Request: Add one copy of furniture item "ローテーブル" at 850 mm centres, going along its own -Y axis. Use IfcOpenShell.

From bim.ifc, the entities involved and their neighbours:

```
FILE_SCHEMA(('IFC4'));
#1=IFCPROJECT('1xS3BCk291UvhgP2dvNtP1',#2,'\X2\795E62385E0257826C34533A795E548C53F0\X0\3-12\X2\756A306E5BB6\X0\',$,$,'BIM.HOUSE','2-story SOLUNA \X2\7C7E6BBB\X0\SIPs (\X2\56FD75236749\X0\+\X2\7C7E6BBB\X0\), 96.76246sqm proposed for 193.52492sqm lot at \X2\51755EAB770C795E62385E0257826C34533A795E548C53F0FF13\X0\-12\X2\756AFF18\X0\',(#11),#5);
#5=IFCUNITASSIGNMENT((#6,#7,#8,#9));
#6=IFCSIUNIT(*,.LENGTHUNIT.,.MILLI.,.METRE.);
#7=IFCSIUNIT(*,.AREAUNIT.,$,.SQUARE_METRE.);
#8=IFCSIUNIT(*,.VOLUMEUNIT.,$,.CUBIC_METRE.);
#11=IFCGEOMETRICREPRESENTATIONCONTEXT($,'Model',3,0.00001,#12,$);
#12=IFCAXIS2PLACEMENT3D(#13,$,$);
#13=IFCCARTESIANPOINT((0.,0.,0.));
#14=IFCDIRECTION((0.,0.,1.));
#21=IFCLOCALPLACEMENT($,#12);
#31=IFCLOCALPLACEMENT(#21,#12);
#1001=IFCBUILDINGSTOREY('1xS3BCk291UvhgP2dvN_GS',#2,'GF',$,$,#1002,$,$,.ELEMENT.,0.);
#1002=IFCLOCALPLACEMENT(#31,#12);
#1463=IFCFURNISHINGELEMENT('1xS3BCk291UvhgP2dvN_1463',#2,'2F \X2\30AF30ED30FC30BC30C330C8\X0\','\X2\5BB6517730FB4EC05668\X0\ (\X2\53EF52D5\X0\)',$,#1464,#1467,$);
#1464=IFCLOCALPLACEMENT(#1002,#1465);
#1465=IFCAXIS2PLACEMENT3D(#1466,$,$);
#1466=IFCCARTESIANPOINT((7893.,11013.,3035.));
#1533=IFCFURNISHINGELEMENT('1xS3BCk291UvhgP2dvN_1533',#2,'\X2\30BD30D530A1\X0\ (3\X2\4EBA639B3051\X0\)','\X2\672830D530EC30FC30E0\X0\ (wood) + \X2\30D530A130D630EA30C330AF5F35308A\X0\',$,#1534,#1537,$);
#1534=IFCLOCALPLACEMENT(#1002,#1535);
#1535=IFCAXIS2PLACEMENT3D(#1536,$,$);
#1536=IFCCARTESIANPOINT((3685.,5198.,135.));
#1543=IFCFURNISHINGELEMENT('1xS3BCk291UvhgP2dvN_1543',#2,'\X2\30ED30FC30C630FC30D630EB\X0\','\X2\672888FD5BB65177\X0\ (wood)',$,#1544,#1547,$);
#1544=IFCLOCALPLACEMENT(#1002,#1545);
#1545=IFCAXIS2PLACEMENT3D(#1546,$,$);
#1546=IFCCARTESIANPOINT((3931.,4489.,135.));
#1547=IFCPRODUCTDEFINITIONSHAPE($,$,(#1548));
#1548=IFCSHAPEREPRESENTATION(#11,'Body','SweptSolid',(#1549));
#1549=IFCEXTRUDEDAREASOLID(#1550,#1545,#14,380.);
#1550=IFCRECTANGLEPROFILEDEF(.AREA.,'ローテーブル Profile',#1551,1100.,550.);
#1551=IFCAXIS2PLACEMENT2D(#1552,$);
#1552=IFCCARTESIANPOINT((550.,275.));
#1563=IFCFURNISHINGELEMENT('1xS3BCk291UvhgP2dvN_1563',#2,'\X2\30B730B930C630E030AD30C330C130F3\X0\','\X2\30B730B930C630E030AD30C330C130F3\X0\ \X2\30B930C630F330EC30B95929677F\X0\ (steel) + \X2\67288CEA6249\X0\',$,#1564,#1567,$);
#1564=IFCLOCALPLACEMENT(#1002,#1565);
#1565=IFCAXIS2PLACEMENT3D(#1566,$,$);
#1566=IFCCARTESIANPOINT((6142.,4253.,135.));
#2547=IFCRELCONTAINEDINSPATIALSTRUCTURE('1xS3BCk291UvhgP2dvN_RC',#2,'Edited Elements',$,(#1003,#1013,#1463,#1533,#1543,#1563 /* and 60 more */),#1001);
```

```python
import ifcopenshell
import ifcopenshell.api.geometry
import ifcopenshell.api.root
import ifcopenshell.util.element
import ifcopenshell.util.placement
import ifcopenshell.util.unit

model = ifcopenshell.open("bim.ifc")
unit_scale = ifcopenshell.util.unit.calculate_unit_scale(model)


def reuse_history(source, copy):
    """copy_class also copies each property set's owner history, people and application; keep the originals."""
    for rel in copy.IsDefinedBy:
        if rel.is_a("IfcRelDefinesByProperties") and (history := rel.RelatingPropertyDefinition.OwnerHistory):
            rel.RelatingPropertyDefinition.OwnerHistory = source.OwnerHistory
            ifcopenshell.util.element.remove_deep2(model, history)


source = model.by_id(1543)
base = ifcopenshell.util.placement.get_local_placement(source.ObjectPlacement)
step = -base[:3, 1] * 0.85 / unit_scale

for i in range(1, 2):
    copy = ifcopenshell.api.root.copy_class(model, product=source)
    copy.Representation = ifcopenshell.util.element.copy_deep(
        model, source.Representation, exclude=["IfcGeometricRepresentationContext", "IfcRepresentationMap"]
    )
    reuse_history(source, copy)
    matrix = base.copy()
    matrix[:3, 3] += i * step
    print("added at", matrix[:3, 3].round(3) + 0.0)
    ifcopenshell.api.geometry.edit_object_placement(model, product=copy, matrix=matrix, is_si=False)

model.write("bim_rev.ifc")
```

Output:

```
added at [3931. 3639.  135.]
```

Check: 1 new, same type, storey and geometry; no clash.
